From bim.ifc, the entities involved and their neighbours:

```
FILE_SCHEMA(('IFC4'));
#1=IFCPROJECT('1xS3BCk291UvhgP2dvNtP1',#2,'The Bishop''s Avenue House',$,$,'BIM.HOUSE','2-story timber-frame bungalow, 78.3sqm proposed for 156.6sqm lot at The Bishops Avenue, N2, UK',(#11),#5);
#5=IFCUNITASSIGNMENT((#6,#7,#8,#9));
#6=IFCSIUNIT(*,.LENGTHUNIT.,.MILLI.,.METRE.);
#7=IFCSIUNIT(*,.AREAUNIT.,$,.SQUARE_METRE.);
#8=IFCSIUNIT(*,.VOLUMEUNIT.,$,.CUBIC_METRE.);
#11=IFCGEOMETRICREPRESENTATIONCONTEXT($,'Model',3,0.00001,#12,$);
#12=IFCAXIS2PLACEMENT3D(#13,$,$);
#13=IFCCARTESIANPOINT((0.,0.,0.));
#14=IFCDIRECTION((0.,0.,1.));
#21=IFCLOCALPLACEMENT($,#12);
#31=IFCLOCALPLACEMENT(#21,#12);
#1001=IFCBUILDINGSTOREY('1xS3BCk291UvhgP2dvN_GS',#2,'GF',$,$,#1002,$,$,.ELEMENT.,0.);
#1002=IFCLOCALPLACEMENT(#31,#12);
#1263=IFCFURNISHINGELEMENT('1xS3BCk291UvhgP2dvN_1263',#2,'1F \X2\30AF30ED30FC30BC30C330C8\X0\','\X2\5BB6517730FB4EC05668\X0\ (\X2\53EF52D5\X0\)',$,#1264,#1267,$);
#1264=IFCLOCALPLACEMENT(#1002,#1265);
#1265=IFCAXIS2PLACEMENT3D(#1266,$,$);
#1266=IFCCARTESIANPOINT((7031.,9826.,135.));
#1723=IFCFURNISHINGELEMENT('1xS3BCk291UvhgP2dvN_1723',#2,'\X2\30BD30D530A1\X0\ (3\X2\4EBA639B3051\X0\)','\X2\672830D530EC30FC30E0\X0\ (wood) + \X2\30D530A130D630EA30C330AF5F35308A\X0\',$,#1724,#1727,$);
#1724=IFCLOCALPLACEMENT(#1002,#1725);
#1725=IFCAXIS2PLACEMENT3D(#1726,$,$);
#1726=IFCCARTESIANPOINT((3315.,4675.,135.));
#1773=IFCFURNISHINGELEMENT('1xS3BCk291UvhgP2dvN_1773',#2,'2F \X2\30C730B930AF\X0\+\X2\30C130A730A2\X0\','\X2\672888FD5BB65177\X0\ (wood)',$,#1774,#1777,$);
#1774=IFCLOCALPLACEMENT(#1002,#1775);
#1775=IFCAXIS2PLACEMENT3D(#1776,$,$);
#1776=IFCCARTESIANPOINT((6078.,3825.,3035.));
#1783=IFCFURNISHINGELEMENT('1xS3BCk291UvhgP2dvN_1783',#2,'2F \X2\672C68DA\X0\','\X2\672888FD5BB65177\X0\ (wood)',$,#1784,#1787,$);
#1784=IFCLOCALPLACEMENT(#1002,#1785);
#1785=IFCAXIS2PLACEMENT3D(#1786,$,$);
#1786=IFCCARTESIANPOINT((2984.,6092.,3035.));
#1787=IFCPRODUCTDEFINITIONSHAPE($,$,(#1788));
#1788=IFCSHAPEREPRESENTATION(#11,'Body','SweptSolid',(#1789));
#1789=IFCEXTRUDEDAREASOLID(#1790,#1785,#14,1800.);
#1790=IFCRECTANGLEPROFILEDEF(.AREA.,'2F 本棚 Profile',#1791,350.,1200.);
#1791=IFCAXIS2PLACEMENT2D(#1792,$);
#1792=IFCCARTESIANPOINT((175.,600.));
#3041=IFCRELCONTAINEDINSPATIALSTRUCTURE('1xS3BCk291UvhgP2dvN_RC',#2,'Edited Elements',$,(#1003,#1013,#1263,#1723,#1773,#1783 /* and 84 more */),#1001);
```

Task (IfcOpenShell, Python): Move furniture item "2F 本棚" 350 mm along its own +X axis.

```python
import ifcopenshell
import ifcopenshell.api.geometry
import ifcopenshell.util.placement
import ifcopenshell.util.unit

model = ifcopenshell.open("bim.ifc")
unit_scale = ifcopenshell.util.unit.calculate_unit_scale(model)

item = model.by_guid("1xS3BCk291UvhgP2dvN_1783")
matrix = ifcopenshell.util.placement.get_local_placement(item.ObjectPlacement)
matrix[:3, 3] += matrix[:3, 0] * 0.35 / unit_scale
ifcopenshell.api.geometry.edit_object_placement(model, product=item, matrix=matrix, is_si=False)

print(ifcopenshell.util.placement.get_local_placement(item.ObjectPlacement).round(3) + 0.0)

model.write("bim_updated.ifc")
```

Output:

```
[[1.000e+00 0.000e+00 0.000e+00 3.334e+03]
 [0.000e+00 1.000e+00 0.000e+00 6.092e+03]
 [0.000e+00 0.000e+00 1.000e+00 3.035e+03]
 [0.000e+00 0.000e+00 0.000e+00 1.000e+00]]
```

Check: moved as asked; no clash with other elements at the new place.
